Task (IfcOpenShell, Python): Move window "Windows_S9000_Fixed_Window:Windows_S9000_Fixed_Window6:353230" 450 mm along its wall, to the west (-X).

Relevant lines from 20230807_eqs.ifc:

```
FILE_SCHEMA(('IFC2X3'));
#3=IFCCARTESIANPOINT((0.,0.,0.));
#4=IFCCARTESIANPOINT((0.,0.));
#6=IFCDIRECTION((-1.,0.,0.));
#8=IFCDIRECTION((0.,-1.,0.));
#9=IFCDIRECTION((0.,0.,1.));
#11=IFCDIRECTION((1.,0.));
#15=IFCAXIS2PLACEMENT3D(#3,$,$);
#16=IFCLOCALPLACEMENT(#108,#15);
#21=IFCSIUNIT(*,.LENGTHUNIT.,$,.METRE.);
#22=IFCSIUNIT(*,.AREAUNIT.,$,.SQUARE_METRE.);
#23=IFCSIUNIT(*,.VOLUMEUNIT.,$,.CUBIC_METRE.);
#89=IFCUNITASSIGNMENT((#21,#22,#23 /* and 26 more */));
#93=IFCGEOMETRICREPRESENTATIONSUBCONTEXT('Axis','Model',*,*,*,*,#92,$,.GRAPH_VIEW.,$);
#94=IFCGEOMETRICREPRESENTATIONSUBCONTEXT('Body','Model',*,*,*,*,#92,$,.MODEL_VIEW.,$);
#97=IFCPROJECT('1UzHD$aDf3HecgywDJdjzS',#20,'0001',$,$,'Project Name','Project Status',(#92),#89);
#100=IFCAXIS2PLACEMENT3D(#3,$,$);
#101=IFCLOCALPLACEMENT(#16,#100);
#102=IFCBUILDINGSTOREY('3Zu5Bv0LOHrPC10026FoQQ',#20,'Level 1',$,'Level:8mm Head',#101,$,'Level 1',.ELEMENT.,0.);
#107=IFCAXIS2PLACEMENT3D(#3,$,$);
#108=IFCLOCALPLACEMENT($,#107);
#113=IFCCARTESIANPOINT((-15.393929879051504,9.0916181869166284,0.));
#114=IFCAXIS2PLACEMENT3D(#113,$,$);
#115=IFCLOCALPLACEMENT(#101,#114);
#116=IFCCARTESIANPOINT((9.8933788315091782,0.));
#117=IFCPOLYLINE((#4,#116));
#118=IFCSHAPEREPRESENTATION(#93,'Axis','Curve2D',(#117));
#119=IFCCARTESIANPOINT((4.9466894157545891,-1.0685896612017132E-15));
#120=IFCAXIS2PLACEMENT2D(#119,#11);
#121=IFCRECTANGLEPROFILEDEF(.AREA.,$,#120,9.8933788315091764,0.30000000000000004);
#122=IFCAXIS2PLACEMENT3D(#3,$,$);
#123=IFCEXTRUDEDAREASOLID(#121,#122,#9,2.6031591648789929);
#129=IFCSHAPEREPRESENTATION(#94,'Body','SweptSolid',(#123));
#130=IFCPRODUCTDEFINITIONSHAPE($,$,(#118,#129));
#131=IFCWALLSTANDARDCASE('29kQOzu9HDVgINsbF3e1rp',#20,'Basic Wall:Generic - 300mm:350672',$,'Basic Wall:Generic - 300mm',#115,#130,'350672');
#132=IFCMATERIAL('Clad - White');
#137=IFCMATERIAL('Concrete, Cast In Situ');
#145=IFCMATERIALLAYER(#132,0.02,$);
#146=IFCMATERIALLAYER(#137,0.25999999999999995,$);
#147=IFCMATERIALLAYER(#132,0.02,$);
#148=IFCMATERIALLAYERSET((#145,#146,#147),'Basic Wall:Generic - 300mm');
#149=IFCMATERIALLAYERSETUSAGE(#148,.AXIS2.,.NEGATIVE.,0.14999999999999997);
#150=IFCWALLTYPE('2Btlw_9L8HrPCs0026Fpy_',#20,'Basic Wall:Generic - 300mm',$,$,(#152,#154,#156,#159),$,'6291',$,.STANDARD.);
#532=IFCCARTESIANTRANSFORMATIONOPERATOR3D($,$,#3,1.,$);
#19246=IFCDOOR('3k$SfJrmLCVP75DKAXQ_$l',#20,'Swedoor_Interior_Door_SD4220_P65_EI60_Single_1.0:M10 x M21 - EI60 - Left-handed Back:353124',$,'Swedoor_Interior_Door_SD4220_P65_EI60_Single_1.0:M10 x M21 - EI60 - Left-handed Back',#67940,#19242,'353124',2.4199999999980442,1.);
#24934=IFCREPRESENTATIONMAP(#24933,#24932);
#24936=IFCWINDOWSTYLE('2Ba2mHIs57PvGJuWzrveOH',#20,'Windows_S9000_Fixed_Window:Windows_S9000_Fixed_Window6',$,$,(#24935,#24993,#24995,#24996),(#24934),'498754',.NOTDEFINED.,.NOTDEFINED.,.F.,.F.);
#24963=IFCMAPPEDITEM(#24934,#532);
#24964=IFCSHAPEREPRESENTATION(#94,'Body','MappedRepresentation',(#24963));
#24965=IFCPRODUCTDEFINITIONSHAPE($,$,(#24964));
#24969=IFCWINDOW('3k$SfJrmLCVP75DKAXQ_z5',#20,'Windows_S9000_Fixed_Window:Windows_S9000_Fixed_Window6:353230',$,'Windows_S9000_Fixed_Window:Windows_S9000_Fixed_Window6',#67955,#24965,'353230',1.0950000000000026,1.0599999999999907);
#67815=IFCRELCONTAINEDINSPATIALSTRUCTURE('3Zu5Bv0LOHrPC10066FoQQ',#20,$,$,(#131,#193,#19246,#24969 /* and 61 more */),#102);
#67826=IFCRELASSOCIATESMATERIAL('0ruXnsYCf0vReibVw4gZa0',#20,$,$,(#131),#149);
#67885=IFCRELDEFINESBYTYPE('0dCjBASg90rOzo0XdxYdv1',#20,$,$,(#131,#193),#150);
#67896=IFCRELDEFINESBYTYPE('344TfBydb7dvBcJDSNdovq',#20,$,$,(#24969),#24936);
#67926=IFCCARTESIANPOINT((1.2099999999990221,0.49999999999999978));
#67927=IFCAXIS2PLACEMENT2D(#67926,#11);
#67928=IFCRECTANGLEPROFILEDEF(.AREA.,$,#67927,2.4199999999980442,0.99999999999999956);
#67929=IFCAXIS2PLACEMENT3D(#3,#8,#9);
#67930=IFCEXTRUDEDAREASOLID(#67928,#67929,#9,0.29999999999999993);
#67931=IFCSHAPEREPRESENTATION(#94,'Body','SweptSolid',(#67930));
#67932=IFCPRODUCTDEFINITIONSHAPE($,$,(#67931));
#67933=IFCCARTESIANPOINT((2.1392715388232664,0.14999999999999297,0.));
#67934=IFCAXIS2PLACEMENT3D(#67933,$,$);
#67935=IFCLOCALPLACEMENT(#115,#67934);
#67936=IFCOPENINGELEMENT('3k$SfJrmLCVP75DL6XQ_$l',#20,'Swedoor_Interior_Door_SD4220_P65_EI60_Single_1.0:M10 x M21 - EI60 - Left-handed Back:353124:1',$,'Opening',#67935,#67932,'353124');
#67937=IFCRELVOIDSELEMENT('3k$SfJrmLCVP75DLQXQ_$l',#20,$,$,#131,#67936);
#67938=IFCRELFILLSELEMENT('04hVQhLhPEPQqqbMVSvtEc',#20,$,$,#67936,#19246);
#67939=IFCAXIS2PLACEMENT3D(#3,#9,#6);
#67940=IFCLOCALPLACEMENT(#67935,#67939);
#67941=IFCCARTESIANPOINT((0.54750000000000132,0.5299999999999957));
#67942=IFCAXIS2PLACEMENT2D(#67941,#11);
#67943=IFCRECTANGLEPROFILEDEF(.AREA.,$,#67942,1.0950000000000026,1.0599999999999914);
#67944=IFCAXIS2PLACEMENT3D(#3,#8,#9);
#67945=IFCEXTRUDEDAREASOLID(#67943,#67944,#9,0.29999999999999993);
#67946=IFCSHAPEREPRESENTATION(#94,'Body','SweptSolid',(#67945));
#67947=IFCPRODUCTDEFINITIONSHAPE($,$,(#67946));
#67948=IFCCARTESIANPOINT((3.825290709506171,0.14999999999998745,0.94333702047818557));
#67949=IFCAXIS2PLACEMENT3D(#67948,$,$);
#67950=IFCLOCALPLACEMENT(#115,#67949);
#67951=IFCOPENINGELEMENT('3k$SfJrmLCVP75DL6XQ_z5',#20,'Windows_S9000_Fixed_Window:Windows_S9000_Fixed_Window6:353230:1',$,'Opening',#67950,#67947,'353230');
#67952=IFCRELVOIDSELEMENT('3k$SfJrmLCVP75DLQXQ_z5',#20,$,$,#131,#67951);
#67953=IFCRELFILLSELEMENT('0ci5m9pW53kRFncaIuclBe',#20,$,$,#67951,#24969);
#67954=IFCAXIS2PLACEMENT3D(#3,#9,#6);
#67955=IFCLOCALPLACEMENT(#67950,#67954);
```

```python
import ifcopenshell
import ifcopenshell.api.geometry
import ifcopenshell.util.placement
import ifcopenshell.util.unit

model = ifcopenshell.open("20230807_eqs.ifc")
unit_scale = ifcopenshell.util.unit.calculate_unit_scale(model)

window = model.by_guid("3k$SfJrmLCVP75DKAXQ_z5")
opening = window.FillsVoids[0].RelatingOpeningElement
wall = opening.VoidsElements[0].RelatingBuildingElement

wall_matrix = ifcopenshell.util.placement.get_local_placement(wall.ObjectPlacement)
shift = wall_matrix[:3, 0] * -0.45 / unit_scale
before = ifcopenshell.util.placement.get_local_placement(window.ObjectPlacement)[:3, 3].copy()

# The window is placed relative to its opening, so it follows when the opening moves.
matrix = ifcopenshell.util.placement.get_local_placement(opening.ObjectPlacement)
matrix[:3, 3] += shift
ifcopenshell.api.geometry.edit_object_placement(
    model, product=opening, matrix=matrix, is_si=False, should_transform_children=True
)

after = ifcopenshell.util.placement.get_local_placement(window.ObjectPlacement)[:3, 3]
print("window moved by", (after - before).round(3) + 0.0)

model.write("20230807_eqs_rev.ifc")
```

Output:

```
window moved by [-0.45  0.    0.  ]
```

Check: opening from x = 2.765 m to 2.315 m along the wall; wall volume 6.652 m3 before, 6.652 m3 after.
